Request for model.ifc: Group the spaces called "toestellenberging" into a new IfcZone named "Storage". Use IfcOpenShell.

First a look at what the model holds.

```python
import ifcopenshell

model = ifcopenshell.open("model.ifc")
print(model.schema)
seen = {}
for space in model.by_type("IfcSpace"):
    seen[space.LongName] = seen.get(space.LongName, 0) + 1
for name, count in sorted(seen.items(), key=str):
    print(count, "x", name)
print("zones:", [z.Name for z in model.by_type("IfcZone")][:20])
```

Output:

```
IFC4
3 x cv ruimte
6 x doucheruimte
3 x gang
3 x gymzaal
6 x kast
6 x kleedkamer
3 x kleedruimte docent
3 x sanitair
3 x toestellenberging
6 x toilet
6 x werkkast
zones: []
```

```python
import ifcopenshell
import ifcopenshell.api.group
import ifcopenshell.api.root

model = ifcopenshell.open("model.ifc")

names = {"toestellenberging"}
spaces = [s for s in model.by_type("IfcSpace") if s.LongName in names]

zone = ifcopenshell.api.root.create_entity(model, ifc_class="IfcZone", name="Storage")
ifcopenshell.api.group.assign_group(model, products=spaces, group=zone)
print(len(spaces), "spaces in", zone.Name)

model.write("model_v2.ifc")
```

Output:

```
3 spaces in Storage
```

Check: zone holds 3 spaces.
